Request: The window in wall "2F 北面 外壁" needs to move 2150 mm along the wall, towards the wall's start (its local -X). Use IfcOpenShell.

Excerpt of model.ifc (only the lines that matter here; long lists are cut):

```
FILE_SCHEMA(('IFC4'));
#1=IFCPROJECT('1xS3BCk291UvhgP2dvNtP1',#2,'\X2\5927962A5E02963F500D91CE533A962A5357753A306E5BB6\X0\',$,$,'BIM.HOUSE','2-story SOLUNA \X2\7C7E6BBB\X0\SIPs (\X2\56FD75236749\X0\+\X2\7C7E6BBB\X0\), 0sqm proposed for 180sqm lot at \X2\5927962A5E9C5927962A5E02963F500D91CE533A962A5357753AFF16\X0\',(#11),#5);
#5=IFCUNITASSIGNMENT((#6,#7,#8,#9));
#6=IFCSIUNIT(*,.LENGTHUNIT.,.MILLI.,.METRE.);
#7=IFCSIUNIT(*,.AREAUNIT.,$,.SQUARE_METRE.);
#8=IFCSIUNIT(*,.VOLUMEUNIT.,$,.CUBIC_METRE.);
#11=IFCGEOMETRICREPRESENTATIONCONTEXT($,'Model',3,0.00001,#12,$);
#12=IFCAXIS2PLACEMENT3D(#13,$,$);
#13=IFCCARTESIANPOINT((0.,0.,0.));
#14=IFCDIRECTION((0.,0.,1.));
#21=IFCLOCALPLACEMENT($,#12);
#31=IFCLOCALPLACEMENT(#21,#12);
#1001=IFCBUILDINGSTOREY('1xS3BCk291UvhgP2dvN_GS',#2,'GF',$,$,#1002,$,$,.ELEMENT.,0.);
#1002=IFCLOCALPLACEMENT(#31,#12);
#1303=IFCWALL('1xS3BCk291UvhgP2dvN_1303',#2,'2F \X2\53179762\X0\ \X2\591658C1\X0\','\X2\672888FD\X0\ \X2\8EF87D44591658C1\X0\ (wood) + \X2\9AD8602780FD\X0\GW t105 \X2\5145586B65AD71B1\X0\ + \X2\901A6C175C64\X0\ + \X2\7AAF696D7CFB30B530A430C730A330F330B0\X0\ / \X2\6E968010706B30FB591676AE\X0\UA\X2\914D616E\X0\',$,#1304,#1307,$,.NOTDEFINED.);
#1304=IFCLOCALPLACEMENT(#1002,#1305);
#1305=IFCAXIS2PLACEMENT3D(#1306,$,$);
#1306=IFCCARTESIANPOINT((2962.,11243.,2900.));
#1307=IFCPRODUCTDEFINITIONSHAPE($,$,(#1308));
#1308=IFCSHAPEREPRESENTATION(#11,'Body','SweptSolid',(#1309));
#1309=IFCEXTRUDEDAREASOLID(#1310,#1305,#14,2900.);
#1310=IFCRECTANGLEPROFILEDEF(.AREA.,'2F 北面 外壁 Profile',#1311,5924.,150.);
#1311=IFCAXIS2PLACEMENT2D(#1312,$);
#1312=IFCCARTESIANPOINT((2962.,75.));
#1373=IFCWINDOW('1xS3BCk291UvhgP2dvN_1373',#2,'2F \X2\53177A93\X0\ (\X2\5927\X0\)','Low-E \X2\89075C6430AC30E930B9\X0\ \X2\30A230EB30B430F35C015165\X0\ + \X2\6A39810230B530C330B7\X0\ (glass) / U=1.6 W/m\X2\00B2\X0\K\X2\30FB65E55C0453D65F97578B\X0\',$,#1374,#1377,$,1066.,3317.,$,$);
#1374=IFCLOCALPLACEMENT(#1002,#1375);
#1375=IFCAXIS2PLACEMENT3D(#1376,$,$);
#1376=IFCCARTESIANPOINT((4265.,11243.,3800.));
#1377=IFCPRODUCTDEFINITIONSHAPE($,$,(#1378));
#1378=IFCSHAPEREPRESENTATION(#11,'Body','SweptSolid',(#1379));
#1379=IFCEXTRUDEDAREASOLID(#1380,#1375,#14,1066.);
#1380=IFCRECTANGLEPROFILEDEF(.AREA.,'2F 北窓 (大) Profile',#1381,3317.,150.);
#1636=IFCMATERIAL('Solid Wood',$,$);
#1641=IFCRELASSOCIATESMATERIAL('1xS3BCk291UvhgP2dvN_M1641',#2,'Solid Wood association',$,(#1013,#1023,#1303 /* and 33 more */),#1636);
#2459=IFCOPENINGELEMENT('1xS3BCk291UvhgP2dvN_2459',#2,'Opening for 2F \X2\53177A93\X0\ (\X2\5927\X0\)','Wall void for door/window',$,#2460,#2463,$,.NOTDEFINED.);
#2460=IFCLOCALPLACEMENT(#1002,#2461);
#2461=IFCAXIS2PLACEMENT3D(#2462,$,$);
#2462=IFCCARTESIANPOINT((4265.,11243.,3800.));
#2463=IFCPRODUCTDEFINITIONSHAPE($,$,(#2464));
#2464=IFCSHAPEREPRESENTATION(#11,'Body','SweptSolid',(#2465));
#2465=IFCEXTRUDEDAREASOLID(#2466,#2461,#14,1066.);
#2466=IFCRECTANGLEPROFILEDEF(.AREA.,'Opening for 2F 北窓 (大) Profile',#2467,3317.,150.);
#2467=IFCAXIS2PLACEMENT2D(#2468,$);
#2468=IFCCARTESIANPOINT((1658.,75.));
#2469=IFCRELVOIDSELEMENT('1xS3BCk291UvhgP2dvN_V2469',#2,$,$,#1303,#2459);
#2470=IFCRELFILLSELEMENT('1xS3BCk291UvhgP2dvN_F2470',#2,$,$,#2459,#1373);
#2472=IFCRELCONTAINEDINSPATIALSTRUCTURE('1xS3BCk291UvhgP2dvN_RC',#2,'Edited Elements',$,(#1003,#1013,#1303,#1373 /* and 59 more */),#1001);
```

```python
import ifcopenshell
import ifcopenshell.api.geometry
import ifcopenshell.util.placement

model = ifcopenshell.open("model.ifc")

window = model.by_id(1373)
opening = window.FillsVoids[0].RelatingOpeningElement
wall = opening.VoidsElements[0].RelatingBuildingElement

wall_matrix = ifcopenshell.util.placement.get_local_placement(wall.ObjectPlacement)
shift = wall_matrix[:3, 0] * -2150.0
before = ifcopenshell.util.placement.get_local_placement(window.ObjectPlacement)[:3, 3].copy()

# The window is not placed relative to its opening, so move both.
for product in (opening, window):
    matrix = ifcopenshell.util.placement.get_local_placement(product.ObjectPlacement)
    matrix[:3, 3] += shift
    ifcopenshell.api.geometry.edit_object_placement(model, product=product, matrix=matrix, is_si=False)

after = ifcopenshell.util.placement.get_local_placement(window.ObjectPlacement)[:3, 3]
print("window moved by", (after - before).round(3) + 0.0)

model.write("model_v2.ifc")
```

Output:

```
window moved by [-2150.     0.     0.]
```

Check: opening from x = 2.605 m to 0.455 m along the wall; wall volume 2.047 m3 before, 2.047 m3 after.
